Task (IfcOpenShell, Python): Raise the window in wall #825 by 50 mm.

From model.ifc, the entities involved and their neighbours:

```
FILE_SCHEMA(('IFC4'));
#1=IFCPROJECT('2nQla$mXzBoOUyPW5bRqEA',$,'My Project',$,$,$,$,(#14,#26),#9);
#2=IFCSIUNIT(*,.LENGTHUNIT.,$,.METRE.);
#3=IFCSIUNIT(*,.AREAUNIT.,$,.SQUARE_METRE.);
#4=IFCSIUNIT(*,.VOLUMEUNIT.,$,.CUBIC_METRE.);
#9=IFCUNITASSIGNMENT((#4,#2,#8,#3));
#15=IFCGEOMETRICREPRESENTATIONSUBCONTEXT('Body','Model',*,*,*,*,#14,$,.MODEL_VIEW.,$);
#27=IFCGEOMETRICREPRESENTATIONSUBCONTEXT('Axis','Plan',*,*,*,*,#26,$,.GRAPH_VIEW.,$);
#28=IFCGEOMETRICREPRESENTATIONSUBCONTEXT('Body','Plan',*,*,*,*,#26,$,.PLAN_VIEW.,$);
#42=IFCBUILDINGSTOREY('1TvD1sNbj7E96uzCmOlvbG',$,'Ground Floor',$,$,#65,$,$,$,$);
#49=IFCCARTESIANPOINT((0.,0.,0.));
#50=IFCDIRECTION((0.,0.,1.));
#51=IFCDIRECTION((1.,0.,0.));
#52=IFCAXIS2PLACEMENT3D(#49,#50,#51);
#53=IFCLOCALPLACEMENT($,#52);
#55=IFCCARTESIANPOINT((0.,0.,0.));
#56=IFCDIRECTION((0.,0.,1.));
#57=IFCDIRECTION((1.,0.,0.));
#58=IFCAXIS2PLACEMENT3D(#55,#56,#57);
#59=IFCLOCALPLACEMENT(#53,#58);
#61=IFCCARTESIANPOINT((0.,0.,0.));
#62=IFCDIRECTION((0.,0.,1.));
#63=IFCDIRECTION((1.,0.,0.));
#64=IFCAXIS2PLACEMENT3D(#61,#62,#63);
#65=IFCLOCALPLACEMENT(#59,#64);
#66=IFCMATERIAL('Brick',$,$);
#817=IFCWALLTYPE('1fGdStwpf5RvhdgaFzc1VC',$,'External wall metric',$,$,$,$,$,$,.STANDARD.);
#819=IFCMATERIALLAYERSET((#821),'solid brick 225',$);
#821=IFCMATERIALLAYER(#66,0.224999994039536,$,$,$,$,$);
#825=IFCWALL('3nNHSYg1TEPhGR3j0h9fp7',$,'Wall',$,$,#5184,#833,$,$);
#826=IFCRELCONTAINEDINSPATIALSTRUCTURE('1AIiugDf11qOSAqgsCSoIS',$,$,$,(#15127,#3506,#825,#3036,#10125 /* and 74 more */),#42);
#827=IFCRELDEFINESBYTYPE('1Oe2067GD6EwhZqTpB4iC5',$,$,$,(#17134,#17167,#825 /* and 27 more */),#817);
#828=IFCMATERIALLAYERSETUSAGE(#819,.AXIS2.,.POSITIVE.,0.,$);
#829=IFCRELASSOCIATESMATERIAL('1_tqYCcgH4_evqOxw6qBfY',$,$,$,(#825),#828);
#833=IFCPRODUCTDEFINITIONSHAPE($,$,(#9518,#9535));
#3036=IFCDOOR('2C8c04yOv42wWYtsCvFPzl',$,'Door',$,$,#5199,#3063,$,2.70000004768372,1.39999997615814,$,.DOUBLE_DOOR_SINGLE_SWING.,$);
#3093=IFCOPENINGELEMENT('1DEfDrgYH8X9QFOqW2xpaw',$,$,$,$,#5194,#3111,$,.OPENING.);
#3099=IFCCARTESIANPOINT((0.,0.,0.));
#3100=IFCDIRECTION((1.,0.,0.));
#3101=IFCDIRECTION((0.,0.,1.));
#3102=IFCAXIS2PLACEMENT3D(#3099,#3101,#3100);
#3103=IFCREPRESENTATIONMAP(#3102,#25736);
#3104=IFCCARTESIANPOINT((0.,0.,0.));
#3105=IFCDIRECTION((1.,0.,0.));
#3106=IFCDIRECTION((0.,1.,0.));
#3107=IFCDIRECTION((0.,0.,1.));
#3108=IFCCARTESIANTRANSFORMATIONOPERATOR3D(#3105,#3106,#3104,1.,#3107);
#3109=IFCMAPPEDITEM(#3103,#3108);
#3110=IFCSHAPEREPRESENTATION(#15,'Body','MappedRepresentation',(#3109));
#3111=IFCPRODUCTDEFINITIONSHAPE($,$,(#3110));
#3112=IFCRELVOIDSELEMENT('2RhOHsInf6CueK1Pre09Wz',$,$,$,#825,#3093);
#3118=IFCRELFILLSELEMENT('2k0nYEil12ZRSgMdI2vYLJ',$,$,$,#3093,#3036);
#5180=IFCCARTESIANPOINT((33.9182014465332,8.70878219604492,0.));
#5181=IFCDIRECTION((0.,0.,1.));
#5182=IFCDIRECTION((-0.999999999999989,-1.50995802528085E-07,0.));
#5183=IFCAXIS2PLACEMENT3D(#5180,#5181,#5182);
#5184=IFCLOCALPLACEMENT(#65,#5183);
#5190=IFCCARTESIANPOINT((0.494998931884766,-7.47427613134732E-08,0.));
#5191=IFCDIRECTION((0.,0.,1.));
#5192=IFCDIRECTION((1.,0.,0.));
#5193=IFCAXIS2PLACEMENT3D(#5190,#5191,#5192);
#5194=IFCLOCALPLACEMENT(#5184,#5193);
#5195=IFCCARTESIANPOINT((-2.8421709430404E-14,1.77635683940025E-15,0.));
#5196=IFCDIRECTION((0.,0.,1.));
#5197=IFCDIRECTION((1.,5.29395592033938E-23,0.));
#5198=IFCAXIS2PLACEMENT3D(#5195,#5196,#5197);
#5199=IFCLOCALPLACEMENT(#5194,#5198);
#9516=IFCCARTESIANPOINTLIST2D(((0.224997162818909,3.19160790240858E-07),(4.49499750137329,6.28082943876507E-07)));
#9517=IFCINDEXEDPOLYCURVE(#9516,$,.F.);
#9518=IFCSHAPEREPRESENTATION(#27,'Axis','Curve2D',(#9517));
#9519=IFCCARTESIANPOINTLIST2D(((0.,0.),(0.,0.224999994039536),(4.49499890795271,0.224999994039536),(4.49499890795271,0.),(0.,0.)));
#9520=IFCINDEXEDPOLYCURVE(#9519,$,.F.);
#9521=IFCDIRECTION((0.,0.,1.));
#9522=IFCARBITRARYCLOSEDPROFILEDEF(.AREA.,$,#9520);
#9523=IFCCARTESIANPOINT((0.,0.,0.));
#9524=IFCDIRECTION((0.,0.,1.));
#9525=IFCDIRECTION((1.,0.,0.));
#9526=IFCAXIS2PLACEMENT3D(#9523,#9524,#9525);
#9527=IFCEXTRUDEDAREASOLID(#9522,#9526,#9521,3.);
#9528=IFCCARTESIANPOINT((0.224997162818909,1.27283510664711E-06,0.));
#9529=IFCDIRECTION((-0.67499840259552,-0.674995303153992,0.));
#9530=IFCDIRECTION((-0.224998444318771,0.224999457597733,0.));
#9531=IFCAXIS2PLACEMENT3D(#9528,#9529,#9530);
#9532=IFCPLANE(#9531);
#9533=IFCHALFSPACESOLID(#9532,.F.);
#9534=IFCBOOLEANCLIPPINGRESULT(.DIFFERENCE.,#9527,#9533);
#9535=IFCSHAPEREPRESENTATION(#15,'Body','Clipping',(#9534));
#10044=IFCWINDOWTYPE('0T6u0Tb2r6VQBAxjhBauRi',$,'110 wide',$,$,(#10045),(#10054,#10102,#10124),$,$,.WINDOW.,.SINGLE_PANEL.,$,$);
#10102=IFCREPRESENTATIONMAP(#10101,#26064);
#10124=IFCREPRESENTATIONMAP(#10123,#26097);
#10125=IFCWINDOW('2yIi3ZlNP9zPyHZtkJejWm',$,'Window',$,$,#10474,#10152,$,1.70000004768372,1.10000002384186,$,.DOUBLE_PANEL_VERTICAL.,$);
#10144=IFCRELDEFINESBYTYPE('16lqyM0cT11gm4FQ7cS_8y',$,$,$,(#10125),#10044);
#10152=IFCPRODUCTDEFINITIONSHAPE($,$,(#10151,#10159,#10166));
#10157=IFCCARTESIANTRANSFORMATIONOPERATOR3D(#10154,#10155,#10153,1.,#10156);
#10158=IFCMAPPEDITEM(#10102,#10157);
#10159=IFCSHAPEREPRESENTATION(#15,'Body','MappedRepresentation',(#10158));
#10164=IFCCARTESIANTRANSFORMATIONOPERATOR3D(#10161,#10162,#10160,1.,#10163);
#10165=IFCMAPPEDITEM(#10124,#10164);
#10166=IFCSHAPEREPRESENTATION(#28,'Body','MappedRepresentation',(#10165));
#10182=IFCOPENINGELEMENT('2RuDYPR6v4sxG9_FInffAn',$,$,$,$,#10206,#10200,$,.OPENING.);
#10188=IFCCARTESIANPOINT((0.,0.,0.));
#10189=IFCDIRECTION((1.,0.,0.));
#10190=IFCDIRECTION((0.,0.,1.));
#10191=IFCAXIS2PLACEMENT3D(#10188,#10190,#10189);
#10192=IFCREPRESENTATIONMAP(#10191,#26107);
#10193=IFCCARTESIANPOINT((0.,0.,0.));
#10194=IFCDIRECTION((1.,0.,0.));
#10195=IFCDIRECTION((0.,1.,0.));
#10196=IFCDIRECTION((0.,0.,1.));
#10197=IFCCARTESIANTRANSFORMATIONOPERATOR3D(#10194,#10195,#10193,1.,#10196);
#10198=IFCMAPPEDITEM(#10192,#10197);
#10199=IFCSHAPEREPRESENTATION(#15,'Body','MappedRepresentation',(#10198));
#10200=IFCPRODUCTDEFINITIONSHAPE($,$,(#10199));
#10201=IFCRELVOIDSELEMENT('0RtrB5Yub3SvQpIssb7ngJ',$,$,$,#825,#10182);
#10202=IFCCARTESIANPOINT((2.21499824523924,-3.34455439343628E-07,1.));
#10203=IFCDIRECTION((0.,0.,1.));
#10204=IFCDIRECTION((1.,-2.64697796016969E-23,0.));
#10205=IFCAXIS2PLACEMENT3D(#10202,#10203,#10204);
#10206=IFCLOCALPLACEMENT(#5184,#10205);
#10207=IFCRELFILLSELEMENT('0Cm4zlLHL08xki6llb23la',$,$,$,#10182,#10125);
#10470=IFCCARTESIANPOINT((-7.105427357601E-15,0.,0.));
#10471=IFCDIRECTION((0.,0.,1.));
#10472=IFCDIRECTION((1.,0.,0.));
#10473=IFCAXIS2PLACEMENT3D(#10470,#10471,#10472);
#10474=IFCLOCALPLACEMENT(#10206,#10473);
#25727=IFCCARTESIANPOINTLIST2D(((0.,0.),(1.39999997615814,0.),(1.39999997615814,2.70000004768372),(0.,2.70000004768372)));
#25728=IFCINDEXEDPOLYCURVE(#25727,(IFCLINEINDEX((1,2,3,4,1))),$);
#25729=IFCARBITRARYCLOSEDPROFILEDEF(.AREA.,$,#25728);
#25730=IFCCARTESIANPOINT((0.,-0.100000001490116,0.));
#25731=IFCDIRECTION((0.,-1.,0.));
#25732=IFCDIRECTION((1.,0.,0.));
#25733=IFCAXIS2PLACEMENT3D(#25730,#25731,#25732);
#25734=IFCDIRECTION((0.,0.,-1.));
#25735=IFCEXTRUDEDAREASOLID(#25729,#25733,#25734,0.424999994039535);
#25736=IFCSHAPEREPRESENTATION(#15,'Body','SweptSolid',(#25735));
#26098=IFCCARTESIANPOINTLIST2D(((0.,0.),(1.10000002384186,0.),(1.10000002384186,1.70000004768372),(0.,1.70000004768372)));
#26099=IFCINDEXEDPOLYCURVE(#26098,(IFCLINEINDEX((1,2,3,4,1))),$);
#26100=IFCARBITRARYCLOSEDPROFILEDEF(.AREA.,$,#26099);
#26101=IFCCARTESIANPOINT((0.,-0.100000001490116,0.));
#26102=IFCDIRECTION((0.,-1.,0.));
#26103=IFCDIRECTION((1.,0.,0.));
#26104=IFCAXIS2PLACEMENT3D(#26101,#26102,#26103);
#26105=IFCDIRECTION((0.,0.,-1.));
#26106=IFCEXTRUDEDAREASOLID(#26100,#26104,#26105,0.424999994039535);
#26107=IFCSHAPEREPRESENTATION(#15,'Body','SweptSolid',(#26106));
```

```python
import numpy as np
import ifcopenshell
import ifcopenshell.api.geometry
import ifcopenshell.util.placement
import ifcopenshell.util.unit

model = ifcopenshell.open("model.ifc")
unit_scale = ifcopenshell.util.unit.calculate_unit_scale(model)

window = model.by_guid("2yIi3ZlNP9zPyHZtkJejWm")
opening = window.FillsVoids[0].RelatingOpeningElement
dz = 0.05 / unit_scale

shift = np.array([0.0, 0.0, dz])
# The window is placed relative to its opening, so it follows when the opening moves.
matrix = ifcopenshell.util.placement.get_local_placement(opening.ObjectPlacement)
matrix[:3, 3] += shift
ifcopenshell.api.geometry.edit_object_placement(
    model, product=opening, matrix=matrix, is_si=False, should_transform_children=True
)

print(f"moved by {dz * unit_scale:+.3f} m")

model.write("model_updated.ifc")
```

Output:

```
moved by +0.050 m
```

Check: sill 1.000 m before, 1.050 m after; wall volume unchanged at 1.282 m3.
